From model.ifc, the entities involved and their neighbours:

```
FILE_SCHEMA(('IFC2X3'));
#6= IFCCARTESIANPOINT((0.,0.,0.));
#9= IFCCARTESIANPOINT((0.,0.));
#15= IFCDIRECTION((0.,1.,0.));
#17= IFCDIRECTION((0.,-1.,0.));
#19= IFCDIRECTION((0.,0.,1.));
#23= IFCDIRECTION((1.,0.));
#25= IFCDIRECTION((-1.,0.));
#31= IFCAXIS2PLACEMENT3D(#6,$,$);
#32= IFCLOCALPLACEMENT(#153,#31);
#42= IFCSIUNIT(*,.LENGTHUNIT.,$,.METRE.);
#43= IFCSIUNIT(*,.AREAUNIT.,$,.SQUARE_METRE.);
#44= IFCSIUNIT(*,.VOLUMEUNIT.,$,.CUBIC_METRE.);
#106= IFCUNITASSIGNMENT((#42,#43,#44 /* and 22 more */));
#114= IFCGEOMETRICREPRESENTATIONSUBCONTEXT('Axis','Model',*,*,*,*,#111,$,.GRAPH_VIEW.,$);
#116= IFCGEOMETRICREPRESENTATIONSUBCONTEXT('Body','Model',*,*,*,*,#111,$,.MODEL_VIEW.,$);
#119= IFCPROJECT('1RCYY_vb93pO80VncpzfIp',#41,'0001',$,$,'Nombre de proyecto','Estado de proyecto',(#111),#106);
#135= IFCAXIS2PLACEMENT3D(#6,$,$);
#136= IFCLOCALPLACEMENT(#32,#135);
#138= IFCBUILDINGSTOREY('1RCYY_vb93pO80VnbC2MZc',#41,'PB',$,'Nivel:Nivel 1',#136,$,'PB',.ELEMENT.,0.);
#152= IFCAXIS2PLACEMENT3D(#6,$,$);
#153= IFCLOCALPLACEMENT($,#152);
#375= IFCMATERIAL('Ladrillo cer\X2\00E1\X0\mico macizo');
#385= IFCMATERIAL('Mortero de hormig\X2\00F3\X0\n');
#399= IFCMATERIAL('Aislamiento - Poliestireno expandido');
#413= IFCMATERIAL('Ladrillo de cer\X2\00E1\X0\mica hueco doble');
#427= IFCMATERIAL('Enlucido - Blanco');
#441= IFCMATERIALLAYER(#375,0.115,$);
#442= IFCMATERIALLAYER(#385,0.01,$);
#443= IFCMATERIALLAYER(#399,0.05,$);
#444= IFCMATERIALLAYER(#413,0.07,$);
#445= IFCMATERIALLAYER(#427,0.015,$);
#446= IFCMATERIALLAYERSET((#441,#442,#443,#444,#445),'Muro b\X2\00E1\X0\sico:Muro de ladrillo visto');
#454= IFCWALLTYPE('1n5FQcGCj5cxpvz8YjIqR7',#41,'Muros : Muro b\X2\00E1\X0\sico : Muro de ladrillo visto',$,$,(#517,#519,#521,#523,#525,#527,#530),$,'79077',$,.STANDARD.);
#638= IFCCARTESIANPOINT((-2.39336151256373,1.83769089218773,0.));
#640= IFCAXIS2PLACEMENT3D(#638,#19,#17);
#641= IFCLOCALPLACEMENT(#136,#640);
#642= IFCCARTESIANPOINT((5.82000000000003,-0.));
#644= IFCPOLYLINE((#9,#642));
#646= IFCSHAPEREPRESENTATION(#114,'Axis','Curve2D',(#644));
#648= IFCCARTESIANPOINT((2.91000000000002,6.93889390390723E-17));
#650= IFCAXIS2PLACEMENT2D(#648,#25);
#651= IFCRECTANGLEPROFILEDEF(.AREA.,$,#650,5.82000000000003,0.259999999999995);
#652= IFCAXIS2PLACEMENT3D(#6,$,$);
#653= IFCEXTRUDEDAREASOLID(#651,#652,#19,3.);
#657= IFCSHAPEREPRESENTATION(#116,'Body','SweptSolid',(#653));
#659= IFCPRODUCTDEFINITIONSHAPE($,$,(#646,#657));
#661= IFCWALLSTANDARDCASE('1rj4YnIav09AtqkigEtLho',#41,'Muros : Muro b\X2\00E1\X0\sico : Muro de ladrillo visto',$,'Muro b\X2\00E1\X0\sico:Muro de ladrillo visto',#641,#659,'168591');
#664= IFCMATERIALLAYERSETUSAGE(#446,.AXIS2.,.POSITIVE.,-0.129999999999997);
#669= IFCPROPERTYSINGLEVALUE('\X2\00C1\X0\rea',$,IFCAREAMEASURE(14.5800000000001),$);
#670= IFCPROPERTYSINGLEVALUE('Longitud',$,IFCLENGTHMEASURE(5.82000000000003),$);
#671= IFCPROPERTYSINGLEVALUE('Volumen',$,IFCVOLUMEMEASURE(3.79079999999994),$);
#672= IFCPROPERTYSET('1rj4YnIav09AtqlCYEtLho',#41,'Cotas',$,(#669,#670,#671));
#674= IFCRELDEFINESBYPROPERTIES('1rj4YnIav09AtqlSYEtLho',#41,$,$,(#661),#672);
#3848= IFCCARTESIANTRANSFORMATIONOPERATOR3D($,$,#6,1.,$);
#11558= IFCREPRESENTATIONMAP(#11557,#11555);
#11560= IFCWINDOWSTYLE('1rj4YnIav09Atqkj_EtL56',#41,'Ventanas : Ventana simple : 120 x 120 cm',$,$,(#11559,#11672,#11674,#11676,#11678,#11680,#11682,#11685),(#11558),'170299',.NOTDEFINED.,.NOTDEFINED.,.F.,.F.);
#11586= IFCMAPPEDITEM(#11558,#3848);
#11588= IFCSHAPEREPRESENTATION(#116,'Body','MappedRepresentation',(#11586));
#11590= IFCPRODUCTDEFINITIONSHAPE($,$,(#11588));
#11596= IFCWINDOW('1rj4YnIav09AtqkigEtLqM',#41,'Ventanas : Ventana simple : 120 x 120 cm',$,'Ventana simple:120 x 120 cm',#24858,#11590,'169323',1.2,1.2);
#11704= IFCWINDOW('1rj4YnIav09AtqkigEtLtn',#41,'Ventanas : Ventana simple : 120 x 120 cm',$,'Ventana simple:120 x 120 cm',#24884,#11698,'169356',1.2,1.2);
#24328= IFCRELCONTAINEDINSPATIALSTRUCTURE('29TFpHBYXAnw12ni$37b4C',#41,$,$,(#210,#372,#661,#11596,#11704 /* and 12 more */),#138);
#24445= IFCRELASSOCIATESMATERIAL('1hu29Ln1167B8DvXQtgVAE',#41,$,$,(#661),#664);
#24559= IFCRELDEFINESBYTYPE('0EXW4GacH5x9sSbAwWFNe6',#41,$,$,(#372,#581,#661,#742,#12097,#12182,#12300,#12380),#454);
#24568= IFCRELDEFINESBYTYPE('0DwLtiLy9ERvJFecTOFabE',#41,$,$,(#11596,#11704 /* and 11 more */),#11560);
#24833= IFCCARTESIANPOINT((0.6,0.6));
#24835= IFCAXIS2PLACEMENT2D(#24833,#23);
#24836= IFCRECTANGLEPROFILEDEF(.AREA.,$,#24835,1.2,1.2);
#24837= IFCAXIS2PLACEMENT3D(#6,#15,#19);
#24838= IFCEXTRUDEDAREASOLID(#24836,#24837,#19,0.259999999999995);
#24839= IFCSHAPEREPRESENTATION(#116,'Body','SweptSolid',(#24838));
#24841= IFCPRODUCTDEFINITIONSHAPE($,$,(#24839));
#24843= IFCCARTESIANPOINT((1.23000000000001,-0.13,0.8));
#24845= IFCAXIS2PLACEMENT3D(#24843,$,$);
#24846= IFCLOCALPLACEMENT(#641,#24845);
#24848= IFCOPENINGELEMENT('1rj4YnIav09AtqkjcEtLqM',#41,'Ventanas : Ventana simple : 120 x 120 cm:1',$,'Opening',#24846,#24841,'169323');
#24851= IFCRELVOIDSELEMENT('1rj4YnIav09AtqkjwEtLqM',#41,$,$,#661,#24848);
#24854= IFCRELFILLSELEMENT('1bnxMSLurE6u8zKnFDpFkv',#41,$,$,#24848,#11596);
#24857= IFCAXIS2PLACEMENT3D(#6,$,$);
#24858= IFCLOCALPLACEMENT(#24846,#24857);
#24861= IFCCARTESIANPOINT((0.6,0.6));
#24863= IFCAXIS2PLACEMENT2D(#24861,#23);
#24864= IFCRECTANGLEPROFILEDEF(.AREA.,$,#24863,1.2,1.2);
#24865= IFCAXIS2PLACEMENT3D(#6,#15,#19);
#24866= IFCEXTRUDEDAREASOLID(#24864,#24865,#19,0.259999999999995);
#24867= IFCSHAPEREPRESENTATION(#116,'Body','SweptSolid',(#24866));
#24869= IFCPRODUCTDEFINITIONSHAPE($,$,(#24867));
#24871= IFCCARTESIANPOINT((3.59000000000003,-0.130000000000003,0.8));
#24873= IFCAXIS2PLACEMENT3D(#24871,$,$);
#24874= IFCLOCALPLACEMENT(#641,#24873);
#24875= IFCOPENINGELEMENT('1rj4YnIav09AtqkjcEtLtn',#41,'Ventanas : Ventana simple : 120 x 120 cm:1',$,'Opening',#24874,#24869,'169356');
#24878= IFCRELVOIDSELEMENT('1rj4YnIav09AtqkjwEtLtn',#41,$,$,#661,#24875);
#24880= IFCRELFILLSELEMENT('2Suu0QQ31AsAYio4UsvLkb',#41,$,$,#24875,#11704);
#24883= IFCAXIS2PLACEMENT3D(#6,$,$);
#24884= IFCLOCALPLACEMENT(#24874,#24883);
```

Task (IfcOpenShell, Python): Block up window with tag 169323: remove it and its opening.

```python
import ifcopenshell
import ifcopenshell.api.feature
import ifcopenshell.api.pset
import ifcopenshell.api.root
import ifcopenshell.geom
import ifcopenshell.util.element
import ifcopenshell.util.shape
import ifcopenshell.util.unit

model = ifcopenshell.open("model.ifc")
area_scale = ifcopenshell.util.unit.calculate_unit_scale(model, "AREAUNIT")
volume_scale = ifcopenshell.util.unit.calculate_unit_scale(model, "VOLUMEUNIT")
settings = ifcopenshell.geom.settings()


def volume(element):
    """Net volume in cubic metres, openings subtracted."""
    shape = ifcopenshell.geom.create_shape(settings, element)
    return ifcopenshell.util.shape.get_volume(shape.geometry)


window = model.by_guid("1rj4YnIav09AtqkigEtLqM")
opening = window.FillsVoids[0].RelatingOpeningElement
wall = opening.VoidsElements[0].RelatingBuildingElement
before = volume(wall)

ifcopenshell.api.root.remove_product(model, product=window)
ifcopenshell.api.feature.remove_feature(model, feature=opening)

after = volume(wall)
thickness = 0.26  # wall thickness in metres

# Update the wall's stored quantities.
pset = model.by_id(ifcopenshell.util.element.get_pset(wall, "Cotas", should_inherit=False)["id"])
ifcopenshell.api.pset.edit_pset(model, pset=pset, properties={
    "Área": model.create_entity("IfcAreaMeasure", after / thickness / area_scale),
    "Volumen": model.create_entity("IfcVolumeMeasure", after / volume_scale),
})

print(f"wall volume {before:.3f} -> {after:.3f} m3")

model.write("model_rev.ifc")
```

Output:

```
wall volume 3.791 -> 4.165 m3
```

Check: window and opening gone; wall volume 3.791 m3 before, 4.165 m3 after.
